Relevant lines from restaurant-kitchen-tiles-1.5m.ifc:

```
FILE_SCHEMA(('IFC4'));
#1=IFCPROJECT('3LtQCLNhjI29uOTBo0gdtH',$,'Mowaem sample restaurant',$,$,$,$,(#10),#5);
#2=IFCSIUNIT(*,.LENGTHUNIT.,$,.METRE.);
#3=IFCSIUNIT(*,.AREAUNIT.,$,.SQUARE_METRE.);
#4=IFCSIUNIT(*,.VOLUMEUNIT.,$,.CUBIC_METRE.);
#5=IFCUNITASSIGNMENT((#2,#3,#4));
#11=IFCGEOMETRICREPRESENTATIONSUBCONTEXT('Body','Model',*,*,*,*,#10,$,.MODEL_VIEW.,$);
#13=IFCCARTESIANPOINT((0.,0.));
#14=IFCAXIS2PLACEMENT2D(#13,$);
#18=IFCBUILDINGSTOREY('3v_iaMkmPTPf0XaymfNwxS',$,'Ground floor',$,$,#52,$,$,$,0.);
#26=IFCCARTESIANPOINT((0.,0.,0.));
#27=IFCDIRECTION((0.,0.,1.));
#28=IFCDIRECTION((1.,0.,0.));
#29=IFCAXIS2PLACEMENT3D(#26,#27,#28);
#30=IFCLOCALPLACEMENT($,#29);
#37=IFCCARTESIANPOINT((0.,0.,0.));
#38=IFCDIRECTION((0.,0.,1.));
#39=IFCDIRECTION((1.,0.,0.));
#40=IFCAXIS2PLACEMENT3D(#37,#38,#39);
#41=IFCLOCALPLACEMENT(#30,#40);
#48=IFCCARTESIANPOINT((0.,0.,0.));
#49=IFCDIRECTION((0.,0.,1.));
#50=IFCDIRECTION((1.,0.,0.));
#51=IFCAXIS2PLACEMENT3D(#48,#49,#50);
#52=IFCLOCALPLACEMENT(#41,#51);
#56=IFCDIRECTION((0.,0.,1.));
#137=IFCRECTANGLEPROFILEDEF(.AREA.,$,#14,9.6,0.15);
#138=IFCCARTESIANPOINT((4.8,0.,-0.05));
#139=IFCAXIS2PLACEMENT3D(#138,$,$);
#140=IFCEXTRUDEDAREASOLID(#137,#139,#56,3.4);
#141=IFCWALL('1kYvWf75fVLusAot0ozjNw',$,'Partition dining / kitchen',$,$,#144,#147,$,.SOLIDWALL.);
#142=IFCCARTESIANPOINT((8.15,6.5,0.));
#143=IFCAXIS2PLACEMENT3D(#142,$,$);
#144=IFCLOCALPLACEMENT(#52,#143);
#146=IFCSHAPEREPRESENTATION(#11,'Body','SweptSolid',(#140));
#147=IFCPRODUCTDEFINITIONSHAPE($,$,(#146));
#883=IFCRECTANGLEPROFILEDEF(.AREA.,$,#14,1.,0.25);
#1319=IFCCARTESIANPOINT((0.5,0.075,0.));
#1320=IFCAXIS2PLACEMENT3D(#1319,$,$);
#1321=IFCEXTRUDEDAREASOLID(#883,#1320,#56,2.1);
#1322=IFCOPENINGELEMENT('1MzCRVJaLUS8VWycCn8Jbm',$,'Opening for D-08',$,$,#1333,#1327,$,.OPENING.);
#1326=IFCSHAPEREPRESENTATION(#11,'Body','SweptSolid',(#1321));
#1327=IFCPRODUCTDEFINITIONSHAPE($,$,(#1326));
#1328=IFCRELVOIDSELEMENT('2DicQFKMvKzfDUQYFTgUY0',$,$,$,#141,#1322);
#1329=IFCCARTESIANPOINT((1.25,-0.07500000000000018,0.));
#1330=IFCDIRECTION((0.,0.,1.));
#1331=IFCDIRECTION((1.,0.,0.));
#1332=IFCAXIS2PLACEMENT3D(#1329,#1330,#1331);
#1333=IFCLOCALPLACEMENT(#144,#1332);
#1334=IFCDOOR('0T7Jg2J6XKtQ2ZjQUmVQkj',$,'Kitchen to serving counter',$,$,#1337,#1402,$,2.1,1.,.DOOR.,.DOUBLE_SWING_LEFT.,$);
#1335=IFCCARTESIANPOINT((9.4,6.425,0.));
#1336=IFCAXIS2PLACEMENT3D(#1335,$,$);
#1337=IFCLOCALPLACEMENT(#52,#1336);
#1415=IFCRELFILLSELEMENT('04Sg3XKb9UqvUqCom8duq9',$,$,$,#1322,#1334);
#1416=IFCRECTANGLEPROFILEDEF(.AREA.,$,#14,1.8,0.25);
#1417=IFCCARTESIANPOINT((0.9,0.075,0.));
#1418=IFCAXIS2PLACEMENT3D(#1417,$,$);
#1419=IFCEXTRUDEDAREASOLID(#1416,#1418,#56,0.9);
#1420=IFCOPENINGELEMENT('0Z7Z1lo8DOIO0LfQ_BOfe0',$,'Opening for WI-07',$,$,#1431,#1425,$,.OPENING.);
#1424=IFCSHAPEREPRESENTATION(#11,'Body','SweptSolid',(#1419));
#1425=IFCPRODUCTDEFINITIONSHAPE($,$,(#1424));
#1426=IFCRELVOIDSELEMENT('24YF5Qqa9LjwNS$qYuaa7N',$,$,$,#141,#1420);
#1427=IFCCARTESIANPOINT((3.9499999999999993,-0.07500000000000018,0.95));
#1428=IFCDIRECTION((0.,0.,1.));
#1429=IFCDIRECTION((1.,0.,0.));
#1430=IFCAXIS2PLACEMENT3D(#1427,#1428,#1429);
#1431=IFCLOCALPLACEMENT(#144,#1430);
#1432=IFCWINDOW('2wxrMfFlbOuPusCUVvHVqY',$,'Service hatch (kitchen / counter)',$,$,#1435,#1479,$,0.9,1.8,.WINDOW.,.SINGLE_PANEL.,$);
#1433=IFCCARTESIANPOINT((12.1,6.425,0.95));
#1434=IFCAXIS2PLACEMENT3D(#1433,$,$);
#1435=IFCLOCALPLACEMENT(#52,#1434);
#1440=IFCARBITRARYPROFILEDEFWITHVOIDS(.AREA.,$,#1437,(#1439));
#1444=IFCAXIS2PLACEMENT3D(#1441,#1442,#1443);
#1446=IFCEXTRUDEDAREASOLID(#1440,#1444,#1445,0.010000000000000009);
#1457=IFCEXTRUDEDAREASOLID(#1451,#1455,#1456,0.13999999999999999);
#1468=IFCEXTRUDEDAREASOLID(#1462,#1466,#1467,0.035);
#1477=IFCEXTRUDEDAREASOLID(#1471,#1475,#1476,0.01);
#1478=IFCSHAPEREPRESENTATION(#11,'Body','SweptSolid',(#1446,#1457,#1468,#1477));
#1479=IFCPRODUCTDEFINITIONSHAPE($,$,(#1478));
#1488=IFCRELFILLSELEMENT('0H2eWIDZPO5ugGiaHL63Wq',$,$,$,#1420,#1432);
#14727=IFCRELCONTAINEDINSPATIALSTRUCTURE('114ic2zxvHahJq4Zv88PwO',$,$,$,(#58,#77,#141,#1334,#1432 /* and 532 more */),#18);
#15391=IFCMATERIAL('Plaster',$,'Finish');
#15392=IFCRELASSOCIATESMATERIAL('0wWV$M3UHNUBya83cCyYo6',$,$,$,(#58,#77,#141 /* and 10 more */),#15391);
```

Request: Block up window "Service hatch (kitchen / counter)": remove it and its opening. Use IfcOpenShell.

```python
import ifcopenshell
import ifcopenshell.api.feature
import ifcopenshell.api.root
import ifcopenshell.geom
import ifcopenshell.util.shape

model = ifcopenshell.open("restaurant-kitchen-tiles-1.5m.ifc")
settings = ifcopenshell.geom.settings()


def volume(element):
    """Net volume in cubic metres, openings subtracted."""
    shape = ifcopenshell.geom.create_shape(settings, element)
    return ifcopenshell.util.shape.get_volume(shape.geometry)


window = model.by_id(1432)
opening = window.FillsVoids[0].RelatingOpeningElement
wall = opening.VoidsElements[0].RelatingBuildingElement
before = volume(wall)

ifcopenshell.api.root.remove_product(model, product=window)
ifcopenshell.api.feature.remove_feature(model, feature=opening)

after = volume(wall)

print(f"wall volume {before:.3f} -> {after:.3f} m3")

model.write("restaurant-kitchen-tiles-1.5m_v2.ifc")
```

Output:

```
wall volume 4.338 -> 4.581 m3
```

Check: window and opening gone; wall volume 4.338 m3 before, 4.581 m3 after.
